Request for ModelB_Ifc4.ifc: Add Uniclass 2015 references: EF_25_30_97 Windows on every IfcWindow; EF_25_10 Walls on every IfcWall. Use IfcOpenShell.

First a look at what the model holds.

```python
import ifcopenshell

model = ifcopenshell.open("ModelB_Ifc4.ifc")
print(model.schema)
print("classifications:", [c.Name for c in model.by_type("IfcClassification")])
for ifc_class in ("IfcDoor", "IfcRoof", "IfcStair", "IfcWall", "IfcWindow"):
    print(ifc_class, len(model.by_type(ifc_class)))
```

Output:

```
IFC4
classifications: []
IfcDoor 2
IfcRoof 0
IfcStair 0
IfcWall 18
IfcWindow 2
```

```python
import ifcopenshell
import ifcopenshell.api.classification

model = ifcopenshell.open("ModelB_Ifc4.ifc")

system = ifcopenshell.api.classification.add_classification(model, classification="Uniclass 2015")

codes = {
    "IfcWindow": ("EF_25_30_97", "Windows"),
    "IfcWall": ("EF_25_10", "Walls"),
}
for ifc_class, (code, name) in codes.items():
    products = model.by_type(ifc_class)
    ifcopenshell.api.classification.add_reference(
        model, products=products, classification=system, identification=code, name=name
    )
    print(code, len(products))

model.write("ModelB_Ifc4_edited.ifc")
```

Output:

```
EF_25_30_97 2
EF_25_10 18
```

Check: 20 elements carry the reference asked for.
